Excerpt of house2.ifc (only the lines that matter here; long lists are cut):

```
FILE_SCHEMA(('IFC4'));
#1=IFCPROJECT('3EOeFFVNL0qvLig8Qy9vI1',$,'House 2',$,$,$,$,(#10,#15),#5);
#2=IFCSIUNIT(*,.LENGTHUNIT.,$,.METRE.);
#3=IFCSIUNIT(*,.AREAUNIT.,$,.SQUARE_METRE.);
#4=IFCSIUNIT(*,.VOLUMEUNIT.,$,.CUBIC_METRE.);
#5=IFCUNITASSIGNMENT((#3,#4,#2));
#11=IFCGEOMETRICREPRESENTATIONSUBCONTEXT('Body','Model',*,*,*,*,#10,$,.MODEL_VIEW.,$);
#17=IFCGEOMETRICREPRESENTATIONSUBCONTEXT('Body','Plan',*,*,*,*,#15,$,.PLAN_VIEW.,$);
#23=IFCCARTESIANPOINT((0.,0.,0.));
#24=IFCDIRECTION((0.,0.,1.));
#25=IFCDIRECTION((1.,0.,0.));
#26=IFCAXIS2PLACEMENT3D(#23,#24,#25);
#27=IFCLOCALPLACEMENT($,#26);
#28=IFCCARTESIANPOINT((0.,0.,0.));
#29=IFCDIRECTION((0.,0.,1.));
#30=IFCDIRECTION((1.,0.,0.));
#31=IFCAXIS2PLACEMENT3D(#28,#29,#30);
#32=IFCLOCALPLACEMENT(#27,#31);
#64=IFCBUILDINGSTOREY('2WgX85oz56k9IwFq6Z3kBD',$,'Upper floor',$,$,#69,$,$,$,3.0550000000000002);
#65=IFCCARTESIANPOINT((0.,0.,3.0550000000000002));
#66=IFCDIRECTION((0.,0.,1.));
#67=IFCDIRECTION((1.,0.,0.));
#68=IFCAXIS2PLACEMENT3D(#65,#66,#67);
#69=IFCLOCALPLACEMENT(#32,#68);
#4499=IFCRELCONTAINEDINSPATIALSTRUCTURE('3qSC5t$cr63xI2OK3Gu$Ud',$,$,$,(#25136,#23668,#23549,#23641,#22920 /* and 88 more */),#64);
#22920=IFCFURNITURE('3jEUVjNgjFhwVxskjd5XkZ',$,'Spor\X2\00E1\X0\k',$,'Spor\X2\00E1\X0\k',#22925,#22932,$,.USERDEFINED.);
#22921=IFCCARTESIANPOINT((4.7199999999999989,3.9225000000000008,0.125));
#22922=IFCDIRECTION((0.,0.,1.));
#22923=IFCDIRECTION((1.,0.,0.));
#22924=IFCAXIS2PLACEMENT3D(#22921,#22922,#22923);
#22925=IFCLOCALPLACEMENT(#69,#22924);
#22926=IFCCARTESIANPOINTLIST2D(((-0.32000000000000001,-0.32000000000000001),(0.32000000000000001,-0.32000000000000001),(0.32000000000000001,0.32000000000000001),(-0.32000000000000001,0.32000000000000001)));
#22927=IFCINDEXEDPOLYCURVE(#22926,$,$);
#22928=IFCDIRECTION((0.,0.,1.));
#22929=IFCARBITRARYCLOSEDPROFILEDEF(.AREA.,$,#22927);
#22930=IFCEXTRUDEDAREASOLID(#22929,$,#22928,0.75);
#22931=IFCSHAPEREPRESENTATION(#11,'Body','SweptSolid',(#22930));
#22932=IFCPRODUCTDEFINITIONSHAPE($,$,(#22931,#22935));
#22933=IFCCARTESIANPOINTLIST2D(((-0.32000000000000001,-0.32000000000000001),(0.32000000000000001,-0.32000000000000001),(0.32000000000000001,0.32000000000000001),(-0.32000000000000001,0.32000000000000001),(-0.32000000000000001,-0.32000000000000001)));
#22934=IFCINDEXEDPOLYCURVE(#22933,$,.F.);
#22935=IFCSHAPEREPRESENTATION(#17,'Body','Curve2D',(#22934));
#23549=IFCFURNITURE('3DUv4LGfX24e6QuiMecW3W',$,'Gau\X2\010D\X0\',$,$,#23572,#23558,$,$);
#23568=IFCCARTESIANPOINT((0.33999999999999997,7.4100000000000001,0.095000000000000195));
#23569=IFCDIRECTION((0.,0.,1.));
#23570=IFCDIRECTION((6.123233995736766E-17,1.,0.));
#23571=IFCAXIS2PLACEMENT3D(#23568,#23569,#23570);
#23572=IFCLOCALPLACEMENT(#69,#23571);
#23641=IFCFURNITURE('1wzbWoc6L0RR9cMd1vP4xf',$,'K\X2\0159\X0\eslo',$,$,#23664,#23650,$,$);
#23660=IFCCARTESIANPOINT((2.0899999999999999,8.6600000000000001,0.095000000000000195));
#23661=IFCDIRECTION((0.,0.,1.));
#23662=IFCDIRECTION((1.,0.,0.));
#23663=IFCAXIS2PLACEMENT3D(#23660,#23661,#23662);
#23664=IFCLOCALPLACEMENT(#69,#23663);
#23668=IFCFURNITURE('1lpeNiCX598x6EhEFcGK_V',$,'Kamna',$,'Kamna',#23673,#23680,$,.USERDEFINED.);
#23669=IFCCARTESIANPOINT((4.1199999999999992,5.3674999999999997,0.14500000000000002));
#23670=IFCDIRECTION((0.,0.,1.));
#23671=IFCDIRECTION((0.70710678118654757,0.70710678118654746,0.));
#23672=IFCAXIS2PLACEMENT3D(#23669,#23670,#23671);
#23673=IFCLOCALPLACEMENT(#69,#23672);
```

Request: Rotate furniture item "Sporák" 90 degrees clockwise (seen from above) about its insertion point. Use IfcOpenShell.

```python
import ifcopenshell
import ifcopenshell.api.geometry
import ifcopenshell.util.placement

model = ifcopenshell.open("house2.ifc")

item = model.by_guid("3jEUVjNgjFhwVxskjd5XkZ")
matrix = ifcopenshell.util.placement.get_local_placement(item.ObjectPlacement)
matrix = matrix @ ifcopenshell.util.placement.rotation(-90, "Z")
ifcopenshell.api.geometry.edit_object_placement(model, product=item, matrix=matrix, is_si=False)

print(ifcopenshell.util.placement.get_local_placement(item.ObjectPlacement).round(3) + 0.0)

model.write("house2_v2.ifc")
```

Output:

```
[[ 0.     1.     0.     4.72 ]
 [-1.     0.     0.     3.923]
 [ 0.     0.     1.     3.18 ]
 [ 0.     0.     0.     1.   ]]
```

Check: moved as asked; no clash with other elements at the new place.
